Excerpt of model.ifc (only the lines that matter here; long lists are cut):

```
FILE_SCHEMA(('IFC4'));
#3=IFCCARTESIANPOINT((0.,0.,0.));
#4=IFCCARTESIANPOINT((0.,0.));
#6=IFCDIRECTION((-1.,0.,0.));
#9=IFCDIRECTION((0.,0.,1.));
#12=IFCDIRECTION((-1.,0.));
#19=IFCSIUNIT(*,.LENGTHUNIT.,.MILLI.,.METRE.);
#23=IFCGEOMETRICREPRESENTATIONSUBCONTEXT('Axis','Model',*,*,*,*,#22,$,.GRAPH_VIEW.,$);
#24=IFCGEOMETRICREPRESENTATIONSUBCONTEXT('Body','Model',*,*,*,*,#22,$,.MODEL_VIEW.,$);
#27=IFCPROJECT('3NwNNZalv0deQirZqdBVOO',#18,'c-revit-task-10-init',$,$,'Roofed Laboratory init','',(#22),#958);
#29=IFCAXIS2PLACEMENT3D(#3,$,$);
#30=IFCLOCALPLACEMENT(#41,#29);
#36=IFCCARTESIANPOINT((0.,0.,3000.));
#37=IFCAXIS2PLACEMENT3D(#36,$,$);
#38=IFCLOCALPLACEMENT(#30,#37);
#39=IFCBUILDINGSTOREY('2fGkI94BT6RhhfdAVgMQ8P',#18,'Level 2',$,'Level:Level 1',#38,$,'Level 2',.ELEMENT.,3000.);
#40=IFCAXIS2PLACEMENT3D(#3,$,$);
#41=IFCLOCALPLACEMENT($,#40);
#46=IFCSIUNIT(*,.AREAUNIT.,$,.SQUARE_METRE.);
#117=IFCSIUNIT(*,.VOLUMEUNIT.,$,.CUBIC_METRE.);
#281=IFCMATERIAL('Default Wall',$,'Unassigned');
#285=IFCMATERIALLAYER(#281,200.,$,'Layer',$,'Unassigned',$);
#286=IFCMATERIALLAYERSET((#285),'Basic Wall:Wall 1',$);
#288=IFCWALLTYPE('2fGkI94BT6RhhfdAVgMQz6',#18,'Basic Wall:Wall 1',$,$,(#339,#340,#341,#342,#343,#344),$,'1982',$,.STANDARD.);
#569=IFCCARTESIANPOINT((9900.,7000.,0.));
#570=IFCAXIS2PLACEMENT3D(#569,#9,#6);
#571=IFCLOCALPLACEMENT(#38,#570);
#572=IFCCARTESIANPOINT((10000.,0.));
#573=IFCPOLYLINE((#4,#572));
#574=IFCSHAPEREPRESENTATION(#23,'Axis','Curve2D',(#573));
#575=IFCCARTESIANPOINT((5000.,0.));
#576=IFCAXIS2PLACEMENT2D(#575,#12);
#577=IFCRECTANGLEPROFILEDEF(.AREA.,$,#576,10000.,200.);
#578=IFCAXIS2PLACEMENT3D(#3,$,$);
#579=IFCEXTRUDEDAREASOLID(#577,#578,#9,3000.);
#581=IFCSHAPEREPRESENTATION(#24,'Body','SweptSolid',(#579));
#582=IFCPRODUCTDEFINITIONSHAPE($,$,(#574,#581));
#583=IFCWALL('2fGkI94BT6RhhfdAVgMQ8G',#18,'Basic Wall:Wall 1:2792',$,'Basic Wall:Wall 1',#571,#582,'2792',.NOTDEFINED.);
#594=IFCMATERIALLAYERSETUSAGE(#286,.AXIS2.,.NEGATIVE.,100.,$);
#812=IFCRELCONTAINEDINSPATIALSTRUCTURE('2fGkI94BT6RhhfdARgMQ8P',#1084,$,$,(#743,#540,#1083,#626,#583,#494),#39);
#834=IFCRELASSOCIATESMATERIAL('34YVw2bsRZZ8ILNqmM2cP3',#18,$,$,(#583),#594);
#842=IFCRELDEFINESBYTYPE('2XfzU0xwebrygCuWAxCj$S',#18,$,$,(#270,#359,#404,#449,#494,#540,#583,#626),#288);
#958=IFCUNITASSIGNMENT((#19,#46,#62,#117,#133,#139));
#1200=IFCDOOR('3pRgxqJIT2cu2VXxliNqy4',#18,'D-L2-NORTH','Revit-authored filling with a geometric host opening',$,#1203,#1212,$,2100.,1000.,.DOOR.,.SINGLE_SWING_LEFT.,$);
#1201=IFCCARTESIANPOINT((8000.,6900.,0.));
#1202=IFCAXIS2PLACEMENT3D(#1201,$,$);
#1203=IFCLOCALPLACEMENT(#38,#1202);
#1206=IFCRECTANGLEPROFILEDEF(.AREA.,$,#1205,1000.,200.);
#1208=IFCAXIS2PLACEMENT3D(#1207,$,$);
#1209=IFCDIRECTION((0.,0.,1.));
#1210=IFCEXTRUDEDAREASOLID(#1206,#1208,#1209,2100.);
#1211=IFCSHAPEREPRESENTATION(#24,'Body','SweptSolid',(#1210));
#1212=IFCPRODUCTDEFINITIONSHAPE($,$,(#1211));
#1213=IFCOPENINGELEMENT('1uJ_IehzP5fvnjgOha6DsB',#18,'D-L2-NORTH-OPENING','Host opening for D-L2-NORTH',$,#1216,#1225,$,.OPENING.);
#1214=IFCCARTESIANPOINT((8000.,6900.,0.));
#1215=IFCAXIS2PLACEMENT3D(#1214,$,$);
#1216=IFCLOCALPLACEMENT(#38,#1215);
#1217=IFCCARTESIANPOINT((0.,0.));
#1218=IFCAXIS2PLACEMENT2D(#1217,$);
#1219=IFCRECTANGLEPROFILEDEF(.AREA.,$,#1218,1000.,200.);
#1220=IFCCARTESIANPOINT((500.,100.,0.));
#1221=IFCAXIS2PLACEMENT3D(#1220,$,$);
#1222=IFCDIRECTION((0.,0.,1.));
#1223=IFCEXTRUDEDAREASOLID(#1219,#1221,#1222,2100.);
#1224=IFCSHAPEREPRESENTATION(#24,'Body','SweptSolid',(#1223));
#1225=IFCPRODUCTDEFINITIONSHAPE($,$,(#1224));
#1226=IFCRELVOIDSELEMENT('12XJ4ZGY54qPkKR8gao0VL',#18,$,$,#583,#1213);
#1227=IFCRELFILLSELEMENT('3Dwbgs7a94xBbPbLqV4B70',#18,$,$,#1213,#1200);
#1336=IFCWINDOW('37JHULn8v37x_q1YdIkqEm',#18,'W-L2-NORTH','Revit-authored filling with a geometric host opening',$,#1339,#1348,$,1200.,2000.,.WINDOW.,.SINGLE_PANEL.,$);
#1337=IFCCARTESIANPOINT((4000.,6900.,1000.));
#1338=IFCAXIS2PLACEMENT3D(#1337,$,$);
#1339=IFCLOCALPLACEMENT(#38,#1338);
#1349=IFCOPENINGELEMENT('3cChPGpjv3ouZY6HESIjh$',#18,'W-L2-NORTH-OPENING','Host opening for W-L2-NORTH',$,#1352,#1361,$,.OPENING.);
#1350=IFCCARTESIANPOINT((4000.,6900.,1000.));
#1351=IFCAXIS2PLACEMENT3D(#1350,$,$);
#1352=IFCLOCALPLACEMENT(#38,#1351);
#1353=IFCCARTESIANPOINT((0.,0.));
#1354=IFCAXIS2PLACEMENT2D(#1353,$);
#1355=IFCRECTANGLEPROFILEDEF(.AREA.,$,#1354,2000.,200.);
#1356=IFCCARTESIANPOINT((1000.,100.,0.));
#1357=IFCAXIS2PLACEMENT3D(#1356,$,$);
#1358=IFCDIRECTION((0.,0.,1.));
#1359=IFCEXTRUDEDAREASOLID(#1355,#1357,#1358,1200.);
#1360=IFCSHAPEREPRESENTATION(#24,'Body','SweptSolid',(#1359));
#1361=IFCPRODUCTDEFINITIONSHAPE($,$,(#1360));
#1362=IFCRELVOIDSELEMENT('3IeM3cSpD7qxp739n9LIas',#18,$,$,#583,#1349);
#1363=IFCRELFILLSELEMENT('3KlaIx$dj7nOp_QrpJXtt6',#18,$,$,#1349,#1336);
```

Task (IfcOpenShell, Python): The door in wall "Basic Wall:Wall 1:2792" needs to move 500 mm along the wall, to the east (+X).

```python
import ifcopenshell
import ifcopenshell.api.geometry
import ifcopenshell.util.placement
import ifcopenshell.util.unit

model = ifcopenshell.open("model.ifc")
unit_scale = ifcopenshell.util.unit.calculate_unit_scale(model)

door = model.by_guid("3pRgxqJIT2cu2VXxliNqy4")
opening = door.FillsVoids[0].RelatingOpeningElement
wall = opening.VoidsElements[0].RelatingBuildingElement

wall_matrix = ifcopenshell.util.placement.get_local_placement(wall.ObjectPlacement)
shift = wall_matrix[:3, 0] * -0.5 / unit_scale
before = ifcopenshell.util.placement.get_local_placement(door.ObjectPlacement)[:3, 3].copy()

# The door is not placed relative to its opening, so move both.
for product in (opening, door):
    matrix = ifcopenshell.util.placement.get_local_placement(product.ObjectPlacement)
    matrix[:3, 3] += shift
    ifcopenshell.api.geometry.edit_object_placement(model, product=product, matrix=matrix, is_si=False)

after = ifcopenshell.util.placement.get_local_placement(door.ObjectPlacement)[:3, 3]
print("door moved by", (after - before).round(3) + 0.0)

model.write("model_rev.ifc")
```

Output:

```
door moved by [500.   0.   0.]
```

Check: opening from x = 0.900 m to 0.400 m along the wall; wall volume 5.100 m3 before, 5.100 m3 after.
